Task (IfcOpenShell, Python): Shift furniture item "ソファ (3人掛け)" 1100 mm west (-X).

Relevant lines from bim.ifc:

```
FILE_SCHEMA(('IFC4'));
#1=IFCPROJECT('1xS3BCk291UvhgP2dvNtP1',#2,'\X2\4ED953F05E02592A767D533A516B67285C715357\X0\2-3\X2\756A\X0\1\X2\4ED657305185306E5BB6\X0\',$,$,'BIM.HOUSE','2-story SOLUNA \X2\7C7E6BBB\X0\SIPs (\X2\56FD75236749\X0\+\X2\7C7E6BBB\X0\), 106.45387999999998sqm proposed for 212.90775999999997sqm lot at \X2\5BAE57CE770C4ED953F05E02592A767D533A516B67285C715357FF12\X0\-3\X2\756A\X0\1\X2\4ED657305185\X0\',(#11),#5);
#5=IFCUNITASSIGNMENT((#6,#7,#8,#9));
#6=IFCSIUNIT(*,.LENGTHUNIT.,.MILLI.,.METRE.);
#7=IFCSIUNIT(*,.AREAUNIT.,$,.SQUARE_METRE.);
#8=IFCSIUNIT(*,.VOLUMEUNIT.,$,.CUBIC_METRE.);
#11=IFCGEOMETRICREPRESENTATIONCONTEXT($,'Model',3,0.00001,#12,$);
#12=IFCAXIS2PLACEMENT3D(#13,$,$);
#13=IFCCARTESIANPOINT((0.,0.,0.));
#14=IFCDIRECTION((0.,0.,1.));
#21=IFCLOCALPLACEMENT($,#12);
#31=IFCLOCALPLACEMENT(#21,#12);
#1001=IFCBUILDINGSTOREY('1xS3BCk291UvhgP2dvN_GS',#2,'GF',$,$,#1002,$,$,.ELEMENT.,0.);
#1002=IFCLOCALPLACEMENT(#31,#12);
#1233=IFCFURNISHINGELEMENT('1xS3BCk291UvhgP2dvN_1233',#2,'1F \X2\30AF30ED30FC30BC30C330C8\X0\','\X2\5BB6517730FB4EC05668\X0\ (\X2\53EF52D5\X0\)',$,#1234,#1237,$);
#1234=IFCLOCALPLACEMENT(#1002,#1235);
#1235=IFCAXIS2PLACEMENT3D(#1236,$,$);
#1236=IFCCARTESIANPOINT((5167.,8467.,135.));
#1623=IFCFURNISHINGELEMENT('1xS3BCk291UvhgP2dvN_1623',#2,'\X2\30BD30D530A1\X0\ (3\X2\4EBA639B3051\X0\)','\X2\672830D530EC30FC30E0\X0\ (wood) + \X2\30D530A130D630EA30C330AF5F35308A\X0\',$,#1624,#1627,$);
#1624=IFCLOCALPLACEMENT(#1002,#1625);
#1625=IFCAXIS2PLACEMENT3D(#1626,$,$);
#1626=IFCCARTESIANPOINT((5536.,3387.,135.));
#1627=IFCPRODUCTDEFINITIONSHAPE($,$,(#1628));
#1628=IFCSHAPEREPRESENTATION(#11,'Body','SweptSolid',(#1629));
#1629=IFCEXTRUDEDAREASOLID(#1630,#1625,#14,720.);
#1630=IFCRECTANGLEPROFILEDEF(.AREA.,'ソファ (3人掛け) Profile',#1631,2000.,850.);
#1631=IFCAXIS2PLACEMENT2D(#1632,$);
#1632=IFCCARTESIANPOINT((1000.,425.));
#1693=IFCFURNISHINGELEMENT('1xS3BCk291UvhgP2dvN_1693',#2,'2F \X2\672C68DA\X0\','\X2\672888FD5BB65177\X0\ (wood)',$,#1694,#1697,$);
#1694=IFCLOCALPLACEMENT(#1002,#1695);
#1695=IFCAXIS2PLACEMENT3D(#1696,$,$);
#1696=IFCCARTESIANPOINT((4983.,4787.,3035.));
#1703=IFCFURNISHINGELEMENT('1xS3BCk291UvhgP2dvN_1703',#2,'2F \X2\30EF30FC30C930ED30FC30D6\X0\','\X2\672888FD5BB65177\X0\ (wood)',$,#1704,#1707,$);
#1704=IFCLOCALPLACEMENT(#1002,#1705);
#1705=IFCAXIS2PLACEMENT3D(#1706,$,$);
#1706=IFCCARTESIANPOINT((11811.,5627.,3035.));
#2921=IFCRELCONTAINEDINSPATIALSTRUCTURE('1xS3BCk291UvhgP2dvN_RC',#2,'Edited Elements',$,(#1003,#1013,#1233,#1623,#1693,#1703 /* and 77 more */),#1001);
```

```python
import ifcopenshell
import ifcopenshell.api.geometry
import ifcopenshell.util.placement

model = ifcopenshell.open("bim.ifc")

item = model.by_id(1623)
matrix = ifcopenshell.util.placement.get_local_placement(item.ObjectPlacement)
matrix[0, 3] -= 1100.0
ifcopenshell.api.geometry.edit_object_placement(model, product=item, matrix=matrix, is_si=False)

print(ifcopenshell.util.placement.get_local_placement(item.ObjectPlacement).round(3) + 0.0)

model.write("bim_v2.ifc")
```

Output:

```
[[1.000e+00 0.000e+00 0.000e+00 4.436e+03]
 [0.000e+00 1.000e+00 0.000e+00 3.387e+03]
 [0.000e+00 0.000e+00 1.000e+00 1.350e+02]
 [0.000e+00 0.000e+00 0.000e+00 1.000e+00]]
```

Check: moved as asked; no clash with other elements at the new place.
